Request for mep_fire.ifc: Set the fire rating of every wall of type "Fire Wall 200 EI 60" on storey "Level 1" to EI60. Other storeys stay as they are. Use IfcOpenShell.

First a look at what the model holds.

```python
import ifcopenshell
import ifcopenshell.util.element

model = ifcopenshell.open("mep_fire.ifc")
print(model.schema)
storey = next(s for s in model.by_type("IfcBuildingStorey") if s.Name == "Level 1")
walls = [e for e in ifcopenshell.util.element.get_decomposition(storey) if e.is_a("IfcWall")]
seen = {}
for e in walls:
    element_type = ifcopenshell.util.element.get_type(e)
    key = (element_type.Name if element_type != e and element_type else None, ifcopenshell.util.element.get_pset(e, "Pset_WallCommon", "FireRating"))
    seen[key] = seen.get(key, 0) + 1
for (name, value), count in sorted(seen.items(), key=str):
    print(count, "x", name, "|", value)
```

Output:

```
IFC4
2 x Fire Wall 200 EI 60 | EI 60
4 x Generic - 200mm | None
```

```python
import ifcopenshell
import ifcopenshell.api.pset
import ifcopenshell.util.element

model = ifcopenshell.open("mep_fire.ifc")

storey = next(s for s in model.by_type("IfcBuildingStorey") if s.Name == "Level 1")
walls = [e for e in ifcopenshell.util.element.get_decomposition(storey) if e.is_a("IfcWall")]

count = 0
for e in walls:
    element_type = ifcopenshell.util.element.get_type(e)
    if element_type in (None, e) or element_type.Name != "Fire Wall 200 EI 60":
        continue
    # add_pset returns the element's existing set when there is one.
    pset = ifcopenshell.api.pset.add_pset(model, product=e, name="Pset_WallCommon")
    ifcopenshell.api.pset.edit_pset(model, pset=pset, properties={"FireRating": "EI60"})
    count += 1

print(count, "walls updated")

model.write("mep_fire_updated.ifc")
```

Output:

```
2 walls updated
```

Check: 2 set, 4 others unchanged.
